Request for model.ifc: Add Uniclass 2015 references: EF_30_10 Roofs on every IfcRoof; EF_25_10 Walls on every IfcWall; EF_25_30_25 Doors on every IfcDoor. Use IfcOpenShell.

First a look at what the model holds.

```python
import ifcopenshell

model = ifcopenshell.open("model.ifc")
print(model.schema)
print("classifications:", [c.Name for c in model.by_type("IfcClassification")])
for ifc_class in ("IfcDoor", "IfcRoof", "IfcStair", "IfcWall", "IfcWindow"):
    print(ifc_class, len(model.by_type(ifc_class)))
```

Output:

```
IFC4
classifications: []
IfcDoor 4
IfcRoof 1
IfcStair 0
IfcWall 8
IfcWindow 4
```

```python
import ifcopenshell
import ifcopenshell.api.classification

model = ifcopenshell.open("model.ifc")

system = ifcopenshell.api.classification.add_classification(model, classification="Uniclass 2015")

codes = {
    "IfcRoof": ("EF_30_10", "Roofs"),
    "IfcWall": ("EF_25_10", "Walls"),
    "IfcDoor": ("EF_25_30_25", "Doors"),
}
for ifc_class, (code, name) in codes.items():
    products = model.by_type(ifc_class)
    ifcopenshell.api.classification.add_reference(
        model, products=products, classification=system, identification=code, name=name
    )
    print(code, len(products))

model.write("model-out.ifc")
```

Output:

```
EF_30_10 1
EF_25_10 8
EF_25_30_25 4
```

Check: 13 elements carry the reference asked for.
